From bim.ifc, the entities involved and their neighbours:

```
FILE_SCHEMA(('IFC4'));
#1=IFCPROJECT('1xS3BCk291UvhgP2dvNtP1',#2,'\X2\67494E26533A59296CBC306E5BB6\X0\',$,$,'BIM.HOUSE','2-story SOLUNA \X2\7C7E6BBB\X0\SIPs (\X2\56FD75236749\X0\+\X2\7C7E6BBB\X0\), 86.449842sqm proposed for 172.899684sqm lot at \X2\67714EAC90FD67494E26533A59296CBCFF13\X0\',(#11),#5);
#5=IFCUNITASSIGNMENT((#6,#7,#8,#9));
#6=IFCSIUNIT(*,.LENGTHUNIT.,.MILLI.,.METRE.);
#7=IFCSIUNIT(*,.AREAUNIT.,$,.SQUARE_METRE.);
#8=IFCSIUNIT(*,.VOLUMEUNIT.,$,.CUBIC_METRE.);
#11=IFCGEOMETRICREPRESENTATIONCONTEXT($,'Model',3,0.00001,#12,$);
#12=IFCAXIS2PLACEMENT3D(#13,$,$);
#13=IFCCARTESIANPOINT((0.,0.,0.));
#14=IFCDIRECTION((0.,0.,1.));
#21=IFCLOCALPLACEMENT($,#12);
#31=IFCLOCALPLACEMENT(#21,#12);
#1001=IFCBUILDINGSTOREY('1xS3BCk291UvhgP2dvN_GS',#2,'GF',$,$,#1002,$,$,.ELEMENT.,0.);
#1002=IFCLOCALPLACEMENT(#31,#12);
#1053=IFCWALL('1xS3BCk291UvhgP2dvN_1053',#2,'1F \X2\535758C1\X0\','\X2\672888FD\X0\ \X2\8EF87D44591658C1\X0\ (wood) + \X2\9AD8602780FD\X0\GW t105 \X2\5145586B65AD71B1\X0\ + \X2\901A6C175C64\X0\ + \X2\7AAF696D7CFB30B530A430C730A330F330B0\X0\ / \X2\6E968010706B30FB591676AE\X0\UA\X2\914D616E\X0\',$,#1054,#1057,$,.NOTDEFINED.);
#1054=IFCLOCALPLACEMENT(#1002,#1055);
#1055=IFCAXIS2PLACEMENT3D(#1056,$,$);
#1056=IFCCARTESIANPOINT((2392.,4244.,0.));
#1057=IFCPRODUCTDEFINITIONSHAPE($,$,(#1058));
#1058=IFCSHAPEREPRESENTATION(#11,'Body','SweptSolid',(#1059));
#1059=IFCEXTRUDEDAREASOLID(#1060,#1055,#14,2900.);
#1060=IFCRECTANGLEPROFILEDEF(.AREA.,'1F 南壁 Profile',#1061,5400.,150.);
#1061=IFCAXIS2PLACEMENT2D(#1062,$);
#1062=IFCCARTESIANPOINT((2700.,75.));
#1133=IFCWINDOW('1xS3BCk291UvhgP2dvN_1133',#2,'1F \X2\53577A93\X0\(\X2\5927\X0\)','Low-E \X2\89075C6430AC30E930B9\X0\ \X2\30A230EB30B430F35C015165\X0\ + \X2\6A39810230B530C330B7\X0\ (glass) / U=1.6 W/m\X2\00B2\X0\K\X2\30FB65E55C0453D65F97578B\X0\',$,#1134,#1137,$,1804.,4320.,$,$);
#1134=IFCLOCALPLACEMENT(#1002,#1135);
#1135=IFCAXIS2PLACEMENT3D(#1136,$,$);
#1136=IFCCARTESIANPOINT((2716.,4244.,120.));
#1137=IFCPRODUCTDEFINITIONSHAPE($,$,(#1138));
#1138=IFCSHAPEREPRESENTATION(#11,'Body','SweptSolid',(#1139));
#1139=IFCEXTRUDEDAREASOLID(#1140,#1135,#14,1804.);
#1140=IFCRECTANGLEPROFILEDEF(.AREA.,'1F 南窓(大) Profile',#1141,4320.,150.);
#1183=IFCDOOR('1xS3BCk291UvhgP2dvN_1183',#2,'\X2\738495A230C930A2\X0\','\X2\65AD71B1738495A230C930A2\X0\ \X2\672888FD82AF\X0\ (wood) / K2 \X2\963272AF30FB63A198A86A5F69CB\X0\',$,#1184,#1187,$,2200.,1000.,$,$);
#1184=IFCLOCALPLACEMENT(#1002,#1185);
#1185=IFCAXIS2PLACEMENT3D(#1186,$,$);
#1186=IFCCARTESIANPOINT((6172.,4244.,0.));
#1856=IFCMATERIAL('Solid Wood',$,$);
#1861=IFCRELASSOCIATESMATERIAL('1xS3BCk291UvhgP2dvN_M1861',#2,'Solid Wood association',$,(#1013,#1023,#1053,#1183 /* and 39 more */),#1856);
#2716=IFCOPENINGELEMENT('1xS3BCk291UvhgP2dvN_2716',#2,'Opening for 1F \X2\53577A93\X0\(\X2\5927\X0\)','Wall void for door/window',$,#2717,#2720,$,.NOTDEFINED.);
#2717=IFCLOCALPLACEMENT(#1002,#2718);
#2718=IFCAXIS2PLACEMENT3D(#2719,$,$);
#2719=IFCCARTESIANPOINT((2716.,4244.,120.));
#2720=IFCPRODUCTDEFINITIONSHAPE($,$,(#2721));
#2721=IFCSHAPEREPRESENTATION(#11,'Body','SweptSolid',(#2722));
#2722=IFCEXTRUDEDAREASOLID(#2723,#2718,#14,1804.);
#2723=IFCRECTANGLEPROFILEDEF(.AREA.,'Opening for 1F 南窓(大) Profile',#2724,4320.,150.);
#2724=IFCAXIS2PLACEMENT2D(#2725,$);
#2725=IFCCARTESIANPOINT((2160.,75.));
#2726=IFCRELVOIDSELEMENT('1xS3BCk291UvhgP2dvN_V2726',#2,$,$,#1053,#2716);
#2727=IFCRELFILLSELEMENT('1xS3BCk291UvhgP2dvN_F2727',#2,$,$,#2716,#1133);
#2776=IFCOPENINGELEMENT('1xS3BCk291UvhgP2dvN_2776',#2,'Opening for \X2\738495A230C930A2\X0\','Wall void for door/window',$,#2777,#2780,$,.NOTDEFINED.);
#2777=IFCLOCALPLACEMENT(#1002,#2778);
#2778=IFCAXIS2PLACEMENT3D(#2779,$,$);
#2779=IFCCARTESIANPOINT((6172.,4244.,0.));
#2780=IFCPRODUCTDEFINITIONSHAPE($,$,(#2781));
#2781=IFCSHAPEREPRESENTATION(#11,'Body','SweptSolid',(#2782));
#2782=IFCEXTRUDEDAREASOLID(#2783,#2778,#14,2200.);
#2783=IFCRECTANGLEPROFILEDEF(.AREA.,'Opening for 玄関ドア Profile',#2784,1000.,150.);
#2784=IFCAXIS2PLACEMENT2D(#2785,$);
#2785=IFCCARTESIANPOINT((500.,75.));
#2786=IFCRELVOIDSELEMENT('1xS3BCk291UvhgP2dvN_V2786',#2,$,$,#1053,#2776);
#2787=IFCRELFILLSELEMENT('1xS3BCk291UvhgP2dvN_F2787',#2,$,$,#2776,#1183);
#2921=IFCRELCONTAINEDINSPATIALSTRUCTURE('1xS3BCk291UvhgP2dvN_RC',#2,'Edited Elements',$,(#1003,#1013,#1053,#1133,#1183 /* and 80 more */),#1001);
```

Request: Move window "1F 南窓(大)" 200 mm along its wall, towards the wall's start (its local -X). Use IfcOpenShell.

```python
import ifcopenshell
import ifcopenshell.api.geometry
import ifcopenshell.util.placement

model = ifcopenshell.open("bim.ifc")

window = model.by_guid("1xS3BCk291UvhgP2dvN_1133")
opening = window.FillsVoids[0].RelatingOpeningElement
wall = opening.VoidsElements[0].RelatingBuildingElement

wall_matrix = ifcopenshell.util.placement.get_local_placement(wall.ObjectPlacement)
shift = wall_matrix[:3, 0] * -200.0
before = ifcopenshell.util.placement.get_local_placement(window.ObjectPlacement)[:3, 3].copy()

# The window is not placed relative to its opening, so move both.
for product in (opening, window):
    matrix = ifcopenshell.util.placement.get_local_placement(product.ObjectPlacement)
    matrix[:3, 3] += shift
    ifcopenshell.api.geometry.edit_object_placement(model, product=product, matrix=matrix, is_si=False)

after = ifcopenshell.util.placement.get_local_placement(window.ObjectPlacement)[:3, 3]
print("window moved by", (after - before).round(3) + 0.0)

model.write("bim_updated.ifc")
```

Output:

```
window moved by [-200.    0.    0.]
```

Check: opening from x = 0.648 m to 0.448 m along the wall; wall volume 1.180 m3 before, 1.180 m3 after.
